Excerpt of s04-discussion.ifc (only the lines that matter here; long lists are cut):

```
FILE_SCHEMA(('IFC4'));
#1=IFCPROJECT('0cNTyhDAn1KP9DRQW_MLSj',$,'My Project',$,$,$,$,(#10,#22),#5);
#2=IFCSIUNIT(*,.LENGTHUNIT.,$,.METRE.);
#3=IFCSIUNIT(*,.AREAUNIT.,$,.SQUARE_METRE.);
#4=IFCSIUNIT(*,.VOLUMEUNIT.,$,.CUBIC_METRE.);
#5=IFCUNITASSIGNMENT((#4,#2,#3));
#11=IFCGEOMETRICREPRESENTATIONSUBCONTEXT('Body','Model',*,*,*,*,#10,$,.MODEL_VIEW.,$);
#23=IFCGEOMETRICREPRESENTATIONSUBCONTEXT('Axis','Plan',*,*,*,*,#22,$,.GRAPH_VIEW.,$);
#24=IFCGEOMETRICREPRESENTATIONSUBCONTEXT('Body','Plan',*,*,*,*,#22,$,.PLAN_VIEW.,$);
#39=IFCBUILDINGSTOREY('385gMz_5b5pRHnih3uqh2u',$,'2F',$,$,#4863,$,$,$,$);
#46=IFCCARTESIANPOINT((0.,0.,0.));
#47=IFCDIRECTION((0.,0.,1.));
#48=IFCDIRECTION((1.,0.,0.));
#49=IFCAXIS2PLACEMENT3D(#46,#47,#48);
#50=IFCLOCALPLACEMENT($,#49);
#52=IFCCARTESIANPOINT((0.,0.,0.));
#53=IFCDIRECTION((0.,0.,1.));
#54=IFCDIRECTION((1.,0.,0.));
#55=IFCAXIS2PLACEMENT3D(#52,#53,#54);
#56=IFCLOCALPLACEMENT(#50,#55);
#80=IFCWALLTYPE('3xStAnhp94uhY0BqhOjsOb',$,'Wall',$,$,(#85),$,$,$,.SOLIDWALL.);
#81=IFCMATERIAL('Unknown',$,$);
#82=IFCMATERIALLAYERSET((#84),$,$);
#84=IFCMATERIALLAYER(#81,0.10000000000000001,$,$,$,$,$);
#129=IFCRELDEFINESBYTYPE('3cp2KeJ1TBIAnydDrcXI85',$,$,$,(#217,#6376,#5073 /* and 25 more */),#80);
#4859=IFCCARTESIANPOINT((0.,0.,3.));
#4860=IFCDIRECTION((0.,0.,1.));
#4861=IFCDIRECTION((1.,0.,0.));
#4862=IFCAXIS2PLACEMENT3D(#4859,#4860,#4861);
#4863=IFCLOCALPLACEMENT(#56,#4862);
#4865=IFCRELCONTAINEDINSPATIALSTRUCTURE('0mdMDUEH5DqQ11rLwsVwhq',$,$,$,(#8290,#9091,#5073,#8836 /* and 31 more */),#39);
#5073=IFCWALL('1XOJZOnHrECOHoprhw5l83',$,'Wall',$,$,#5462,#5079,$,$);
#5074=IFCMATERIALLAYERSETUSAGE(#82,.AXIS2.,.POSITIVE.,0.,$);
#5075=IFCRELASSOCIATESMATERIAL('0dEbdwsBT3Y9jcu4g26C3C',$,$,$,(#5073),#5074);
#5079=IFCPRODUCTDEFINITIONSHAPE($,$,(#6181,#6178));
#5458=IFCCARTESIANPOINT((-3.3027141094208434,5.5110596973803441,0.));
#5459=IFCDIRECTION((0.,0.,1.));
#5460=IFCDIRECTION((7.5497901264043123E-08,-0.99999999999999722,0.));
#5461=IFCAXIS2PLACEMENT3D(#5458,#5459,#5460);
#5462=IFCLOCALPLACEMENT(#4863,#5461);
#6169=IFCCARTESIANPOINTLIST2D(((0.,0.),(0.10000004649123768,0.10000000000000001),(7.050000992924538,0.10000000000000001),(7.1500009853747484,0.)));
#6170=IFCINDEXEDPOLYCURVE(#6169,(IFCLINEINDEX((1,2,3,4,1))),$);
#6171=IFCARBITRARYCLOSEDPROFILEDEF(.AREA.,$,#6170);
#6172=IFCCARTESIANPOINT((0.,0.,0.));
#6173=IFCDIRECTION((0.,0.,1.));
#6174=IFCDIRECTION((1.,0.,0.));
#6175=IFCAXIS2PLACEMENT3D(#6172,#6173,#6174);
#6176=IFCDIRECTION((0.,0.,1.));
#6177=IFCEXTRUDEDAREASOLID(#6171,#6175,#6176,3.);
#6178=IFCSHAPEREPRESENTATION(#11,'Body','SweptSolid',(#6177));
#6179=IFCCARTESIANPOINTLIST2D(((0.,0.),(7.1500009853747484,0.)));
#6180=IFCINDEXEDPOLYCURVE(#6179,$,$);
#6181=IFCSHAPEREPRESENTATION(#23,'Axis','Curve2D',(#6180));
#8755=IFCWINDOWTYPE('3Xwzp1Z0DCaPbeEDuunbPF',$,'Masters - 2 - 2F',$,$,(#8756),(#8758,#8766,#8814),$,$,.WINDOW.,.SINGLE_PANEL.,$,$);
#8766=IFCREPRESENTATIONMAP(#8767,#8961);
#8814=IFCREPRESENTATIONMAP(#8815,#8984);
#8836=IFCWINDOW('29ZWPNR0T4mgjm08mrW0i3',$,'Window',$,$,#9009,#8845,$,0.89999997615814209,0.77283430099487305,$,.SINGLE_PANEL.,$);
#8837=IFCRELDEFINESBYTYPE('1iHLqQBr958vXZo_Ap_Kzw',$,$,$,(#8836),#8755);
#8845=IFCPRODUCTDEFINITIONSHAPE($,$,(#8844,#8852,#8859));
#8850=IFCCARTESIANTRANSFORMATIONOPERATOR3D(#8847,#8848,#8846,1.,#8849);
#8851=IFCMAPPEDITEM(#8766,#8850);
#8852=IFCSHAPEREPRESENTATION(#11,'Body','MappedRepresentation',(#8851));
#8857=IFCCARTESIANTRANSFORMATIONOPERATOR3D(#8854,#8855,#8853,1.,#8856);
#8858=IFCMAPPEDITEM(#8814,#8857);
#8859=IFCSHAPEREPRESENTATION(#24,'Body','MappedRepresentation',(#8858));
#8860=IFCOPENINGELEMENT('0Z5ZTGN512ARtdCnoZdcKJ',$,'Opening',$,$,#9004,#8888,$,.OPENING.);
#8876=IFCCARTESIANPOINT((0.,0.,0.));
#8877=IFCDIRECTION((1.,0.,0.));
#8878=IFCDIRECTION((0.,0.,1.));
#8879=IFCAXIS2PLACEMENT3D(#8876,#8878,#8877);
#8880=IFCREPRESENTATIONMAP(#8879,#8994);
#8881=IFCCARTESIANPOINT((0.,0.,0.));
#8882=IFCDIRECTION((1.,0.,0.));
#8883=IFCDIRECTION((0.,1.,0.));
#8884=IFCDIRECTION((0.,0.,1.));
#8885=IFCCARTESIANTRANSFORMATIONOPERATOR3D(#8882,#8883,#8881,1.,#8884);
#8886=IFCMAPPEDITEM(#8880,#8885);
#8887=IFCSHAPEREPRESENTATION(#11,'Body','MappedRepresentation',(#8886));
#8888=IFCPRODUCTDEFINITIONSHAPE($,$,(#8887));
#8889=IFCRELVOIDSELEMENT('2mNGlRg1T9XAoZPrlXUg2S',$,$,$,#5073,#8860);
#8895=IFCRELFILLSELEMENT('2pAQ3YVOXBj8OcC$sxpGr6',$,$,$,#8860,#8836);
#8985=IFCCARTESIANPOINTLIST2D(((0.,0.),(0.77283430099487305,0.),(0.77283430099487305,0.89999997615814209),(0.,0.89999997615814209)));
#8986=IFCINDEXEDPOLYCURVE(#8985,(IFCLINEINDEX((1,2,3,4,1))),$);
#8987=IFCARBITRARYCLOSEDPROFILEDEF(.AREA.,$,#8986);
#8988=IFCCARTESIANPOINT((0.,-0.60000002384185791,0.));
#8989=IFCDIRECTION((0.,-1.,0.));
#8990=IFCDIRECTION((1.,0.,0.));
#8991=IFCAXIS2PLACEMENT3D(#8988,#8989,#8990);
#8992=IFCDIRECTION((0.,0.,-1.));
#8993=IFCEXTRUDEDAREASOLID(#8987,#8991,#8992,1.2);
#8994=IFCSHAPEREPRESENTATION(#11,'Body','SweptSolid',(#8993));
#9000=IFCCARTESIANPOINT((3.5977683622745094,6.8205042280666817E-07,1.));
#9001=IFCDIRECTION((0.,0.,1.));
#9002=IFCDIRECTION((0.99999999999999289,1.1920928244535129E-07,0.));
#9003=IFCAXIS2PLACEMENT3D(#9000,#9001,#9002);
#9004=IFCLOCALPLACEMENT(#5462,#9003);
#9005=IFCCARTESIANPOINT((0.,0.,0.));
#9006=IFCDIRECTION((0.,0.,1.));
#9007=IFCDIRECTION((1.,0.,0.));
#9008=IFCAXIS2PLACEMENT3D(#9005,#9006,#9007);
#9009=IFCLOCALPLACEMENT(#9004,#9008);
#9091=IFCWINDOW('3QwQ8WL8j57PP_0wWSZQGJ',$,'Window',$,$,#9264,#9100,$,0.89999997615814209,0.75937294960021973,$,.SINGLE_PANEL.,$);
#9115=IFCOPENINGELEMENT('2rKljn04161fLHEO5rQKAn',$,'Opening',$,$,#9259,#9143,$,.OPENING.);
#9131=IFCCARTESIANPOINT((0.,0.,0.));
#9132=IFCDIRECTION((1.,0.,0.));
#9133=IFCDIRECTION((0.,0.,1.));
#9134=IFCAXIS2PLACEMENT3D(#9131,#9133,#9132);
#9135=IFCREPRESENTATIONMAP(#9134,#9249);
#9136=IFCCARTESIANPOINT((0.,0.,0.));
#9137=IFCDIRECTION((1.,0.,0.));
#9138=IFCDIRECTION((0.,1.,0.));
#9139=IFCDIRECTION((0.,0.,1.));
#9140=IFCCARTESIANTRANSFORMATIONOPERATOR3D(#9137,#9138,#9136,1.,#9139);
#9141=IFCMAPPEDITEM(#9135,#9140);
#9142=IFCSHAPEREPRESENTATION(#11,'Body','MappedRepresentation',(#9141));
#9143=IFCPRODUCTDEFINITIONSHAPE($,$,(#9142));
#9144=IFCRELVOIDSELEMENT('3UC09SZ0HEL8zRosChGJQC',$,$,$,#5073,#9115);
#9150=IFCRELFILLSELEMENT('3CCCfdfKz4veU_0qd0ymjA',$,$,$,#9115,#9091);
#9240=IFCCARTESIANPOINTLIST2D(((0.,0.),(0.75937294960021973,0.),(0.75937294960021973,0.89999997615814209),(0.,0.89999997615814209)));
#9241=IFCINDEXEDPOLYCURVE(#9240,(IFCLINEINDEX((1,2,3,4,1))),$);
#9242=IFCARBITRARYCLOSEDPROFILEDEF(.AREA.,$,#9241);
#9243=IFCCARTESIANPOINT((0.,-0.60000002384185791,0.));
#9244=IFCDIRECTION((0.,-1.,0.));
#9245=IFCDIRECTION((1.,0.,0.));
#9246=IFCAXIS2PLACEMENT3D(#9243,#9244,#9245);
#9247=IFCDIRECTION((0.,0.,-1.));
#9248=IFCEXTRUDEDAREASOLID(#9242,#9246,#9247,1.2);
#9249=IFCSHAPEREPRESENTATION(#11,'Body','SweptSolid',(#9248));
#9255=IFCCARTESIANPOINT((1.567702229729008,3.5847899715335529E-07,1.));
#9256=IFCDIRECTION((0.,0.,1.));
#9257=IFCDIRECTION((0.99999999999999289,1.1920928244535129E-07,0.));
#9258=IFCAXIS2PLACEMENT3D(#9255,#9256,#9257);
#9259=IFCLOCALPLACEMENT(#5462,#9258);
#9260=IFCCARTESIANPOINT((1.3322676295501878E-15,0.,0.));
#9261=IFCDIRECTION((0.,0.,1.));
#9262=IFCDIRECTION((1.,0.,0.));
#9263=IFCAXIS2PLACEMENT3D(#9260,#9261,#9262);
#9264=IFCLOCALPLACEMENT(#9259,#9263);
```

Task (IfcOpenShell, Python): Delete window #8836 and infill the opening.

```python
import ifcopenshell
import ifcopenshell.api.feature
import ifcopenshell.api.root
import ifcopenshell.geom
import ifcopenshell.util.shape

model = ifcopenshell.open("s04-discussion.ifc")
settings = ifcopenshell.geom.settings()


def volume(element):
    """Net volume in cubic metres, openings subtracted."""
    shape = ifcopenshell.geom.create_shape(settings, element)
    return ifcopenshell.util.shape.get_volume(shape.geometry)


window = model.by_id(8836)
opening = window.FillsVoids[0].RelatingOpeningElement
wall = opening.VoidsElements[0].RelatingBuildingElement
before = volume(wall)

ifcopenshell.api.root.remove_product(model, product=window)
ifcopenshell.api.feature.remove_feature(model, feature=opening)

after = volume(wall)

print(f"wall volume {before:.3f} -> {after:.3f} m3")

model.write("s04-discussion-out.ifc")
```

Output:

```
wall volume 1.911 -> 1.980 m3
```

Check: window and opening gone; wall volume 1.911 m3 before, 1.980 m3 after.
